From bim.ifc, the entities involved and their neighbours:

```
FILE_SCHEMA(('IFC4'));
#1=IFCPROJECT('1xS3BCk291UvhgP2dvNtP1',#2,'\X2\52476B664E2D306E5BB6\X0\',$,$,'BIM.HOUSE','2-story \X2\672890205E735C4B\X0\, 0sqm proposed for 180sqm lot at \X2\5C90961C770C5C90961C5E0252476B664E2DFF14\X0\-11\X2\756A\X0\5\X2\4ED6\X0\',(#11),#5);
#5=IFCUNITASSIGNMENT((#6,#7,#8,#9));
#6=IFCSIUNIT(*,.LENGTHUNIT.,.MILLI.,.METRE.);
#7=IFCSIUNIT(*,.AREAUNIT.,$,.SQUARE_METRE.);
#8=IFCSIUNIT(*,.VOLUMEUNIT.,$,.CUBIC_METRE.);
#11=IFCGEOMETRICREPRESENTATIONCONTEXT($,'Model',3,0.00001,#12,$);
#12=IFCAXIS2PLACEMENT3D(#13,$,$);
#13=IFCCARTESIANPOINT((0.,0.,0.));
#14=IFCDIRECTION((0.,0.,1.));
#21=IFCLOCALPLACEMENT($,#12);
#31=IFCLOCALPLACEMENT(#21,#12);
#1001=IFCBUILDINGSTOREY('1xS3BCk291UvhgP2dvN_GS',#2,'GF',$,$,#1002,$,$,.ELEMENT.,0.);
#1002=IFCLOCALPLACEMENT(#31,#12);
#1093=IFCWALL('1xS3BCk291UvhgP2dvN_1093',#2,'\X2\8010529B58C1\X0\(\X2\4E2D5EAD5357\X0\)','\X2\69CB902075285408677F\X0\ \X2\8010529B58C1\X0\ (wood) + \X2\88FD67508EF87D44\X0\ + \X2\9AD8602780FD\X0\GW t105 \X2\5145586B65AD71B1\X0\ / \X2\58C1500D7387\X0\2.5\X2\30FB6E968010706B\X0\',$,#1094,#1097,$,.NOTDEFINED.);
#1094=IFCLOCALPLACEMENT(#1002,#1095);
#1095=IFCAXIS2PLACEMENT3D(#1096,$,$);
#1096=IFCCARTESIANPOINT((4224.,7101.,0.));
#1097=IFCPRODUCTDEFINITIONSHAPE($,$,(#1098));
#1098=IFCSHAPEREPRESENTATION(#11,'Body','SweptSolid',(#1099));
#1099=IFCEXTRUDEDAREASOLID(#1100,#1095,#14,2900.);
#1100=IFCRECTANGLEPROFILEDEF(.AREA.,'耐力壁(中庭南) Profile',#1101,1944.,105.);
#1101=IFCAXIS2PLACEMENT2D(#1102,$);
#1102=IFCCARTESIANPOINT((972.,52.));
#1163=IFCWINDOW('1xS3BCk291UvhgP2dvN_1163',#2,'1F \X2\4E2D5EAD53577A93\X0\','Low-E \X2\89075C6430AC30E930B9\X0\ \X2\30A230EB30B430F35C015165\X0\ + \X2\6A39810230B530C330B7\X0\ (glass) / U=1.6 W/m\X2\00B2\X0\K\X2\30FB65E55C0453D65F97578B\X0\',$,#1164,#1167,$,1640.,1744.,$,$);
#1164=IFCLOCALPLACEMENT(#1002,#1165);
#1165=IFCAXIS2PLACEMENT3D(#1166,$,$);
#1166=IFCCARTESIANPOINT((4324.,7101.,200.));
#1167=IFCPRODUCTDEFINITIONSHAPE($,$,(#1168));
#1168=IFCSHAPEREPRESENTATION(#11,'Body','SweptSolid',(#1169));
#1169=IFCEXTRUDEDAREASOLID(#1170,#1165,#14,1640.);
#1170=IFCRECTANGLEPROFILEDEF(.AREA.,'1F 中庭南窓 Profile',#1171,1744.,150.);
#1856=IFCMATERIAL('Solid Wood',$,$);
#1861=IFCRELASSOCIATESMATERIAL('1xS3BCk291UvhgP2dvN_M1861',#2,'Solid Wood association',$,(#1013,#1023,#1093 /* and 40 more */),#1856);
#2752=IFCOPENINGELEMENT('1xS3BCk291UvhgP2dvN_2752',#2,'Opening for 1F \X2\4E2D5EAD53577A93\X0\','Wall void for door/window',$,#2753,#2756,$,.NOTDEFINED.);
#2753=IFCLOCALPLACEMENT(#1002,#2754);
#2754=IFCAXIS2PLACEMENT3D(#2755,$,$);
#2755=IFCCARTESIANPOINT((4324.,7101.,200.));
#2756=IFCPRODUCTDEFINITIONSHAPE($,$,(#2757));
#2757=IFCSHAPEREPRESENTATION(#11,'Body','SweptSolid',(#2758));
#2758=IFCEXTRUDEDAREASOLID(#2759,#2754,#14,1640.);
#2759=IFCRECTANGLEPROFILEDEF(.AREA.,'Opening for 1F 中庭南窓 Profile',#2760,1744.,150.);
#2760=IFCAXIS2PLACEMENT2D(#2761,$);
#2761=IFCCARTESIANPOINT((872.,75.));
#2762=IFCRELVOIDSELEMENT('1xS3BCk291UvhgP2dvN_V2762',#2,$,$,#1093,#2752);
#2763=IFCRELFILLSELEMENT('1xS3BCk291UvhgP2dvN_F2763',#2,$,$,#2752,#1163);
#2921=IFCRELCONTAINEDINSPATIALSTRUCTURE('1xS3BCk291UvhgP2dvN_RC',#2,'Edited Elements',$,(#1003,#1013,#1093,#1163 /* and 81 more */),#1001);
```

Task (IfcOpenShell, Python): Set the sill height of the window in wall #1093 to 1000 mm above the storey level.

```python
import numpy as np
import ifcopenshell
import ifcopenshell.api.geometry
import ifcopenshell.geom
import ifcopenshell.util.element
import ifcopenshell.util.placement
import ifcopenshell.util.shape
import ifcopenshell.util.unit

model = ifcopenshell.open("bim.ifc")
unit_scale = ifcopenshell.util.unit.calculate_unit_scale(model)

window = model.by_guid("1xS3BCk291UvhgP2dvN_1163")
opening = window.FillsVoids[0].RelatingOpeningElement
storey = ifcopenshell.util.element.get_container(window, ifc_class="IfcBuildingStorey")
level = ifcopenshell.util.placement.get_local_placement(storey.ObjectPlacement)[2, 3]

# The opening's origin need not be at the sill, so measure its lowest point.
shape = ifcopenshell.geom.create_shape(ifcopenshell.geom.settings(), opening)
bottom = ifcopenshell.util.shape.get_shape_bottom_elevation(shape, shape.geometry) / unit_scale
dz = level + 1 / unit_scale - bottom

shift = np.array([0.0, 0.0, dz])
# The window is not placed relative to its opening, so move both.
for product in (opening, window):
    matrix = ifcopenshell.util.placement.get_local_placement(product.ObjectPlacement)
    matrix[:3, 3] += shift
    ifcopenshell.api.geometry.edit_object_placement(model, product=product, matrix=matrix, is_si=False)

print(f"moved by {dz * unit_scale:+.3f} m")

model.write("bim-out.ifc")
```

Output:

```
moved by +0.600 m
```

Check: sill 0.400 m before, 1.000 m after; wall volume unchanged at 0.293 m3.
